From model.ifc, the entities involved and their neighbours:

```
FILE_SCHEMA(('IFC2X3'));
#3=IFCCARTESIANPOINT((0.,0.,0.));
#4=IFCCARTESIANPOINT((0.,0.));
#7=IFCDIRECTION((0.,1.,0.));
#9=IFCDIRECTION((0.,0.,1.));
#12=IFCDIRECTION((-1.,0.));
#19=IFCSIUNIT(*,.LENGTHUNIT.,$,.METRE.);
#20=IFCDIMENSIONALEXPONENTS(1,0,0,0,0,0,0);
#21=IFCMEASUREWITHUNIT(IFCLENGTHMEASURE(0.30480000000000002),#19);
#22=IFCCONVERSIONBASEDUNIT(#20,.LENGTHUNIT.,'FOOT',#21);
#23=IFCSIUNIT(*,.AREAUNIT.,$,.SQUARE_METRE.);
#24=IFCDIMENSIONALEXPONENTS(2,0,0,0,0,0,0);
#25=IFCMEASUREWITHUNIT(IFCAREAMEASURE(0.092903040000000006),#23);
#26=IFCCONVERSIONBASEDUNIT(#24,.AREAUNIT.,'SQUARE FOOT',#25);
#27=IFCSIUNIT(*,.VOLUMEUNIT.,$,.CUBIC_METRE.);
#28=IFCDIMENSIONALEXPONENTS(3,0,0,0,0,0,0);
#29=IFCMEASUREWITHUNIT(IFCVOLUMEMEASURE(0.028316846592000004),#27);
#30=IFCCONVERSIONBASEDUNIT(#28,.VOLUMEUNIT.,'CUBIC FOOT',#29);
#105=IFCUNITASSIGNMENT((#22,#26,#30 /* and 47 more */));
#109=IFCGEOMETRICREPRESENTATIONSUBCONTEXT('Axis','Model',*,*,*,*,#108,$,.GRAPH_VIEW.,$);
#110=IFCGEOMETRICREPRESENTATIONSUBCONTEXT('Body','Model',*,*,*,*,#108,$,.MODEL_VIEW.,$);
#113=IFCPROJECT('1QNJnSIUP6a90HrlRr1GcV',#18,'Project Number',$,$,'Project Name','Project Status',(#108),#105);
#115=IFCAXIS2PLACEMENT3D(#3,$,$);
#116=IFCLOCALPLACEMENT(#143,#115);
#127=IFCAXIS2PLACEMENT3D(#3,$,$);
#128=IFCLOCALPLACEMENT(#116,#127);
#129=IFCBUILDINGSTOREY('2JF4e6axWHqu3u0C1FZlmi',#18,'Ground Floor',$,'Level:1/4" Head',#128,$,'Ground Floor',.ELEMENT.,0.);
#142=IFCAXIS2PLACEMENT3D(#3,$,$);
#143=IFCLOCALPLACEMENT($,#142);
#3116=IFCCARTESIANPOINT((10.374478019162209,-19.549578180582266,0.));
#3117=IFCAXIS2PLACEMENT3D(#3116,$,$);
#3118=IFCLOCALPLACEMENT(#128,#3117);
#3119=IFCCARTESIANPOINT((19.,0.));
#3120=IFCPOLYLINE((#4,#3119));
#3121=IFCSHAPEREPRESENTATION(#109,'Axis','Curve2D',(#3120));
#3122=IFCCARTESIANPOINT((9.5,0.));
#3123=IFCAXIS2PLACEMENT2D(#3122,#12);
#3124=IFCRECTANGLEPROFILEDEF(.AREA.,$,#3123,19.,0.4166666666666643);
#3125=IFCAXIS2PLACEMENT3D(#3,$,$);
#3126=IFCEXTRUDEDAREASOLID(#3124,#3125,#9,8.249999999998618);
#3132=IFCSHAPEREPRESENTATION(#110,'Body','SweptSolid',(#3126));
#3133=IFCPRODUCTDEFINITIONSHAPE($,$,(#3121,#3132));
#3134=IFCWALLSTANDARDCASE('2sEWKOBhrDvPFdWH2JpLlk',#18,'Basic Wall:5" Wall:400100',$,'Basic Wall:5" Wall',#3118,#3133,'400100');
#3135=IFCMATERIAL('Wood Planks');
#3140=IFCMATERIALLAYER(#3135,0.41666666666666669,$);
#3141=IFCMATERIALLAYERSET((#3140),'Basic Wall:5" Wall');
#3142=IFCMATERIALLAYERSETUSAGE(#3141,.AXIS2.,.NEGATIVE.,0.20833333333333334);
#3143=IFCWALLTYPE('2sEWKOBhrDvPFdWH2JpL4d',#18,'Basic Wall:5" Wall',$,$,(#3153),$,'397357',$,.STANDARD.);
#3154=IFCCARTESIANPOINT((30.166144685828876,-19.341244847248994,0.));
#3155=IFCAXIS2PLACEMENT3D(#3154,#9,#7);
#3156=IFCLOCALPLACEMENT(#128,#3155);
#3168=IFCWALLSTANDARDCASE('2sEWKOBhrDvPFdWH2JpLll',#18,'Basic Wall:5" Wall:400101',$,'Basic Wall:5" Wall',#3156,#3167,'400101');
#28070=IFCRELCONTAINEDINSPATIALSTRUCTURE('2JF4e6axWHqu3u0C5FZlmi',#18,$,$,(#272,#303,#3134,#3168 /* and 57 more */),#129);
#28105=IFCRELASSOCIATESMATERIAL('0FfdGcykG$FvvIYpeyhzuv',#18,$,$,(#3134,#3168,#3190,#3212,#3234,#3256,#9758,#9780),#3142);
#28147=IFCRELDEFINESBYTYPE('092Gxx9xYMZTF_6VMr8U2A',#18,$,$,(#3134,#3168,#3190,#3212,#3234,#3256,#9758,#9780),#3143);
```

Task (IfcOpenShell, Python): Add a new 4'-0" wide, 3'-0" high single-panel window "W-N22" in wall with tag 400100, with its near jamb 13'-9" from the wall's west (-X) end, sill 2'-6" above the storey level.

```python
import numpy as np
import ifcopenshell
import ifcopenshell.api.feature
import ifcopenshell.api.geometry
import ifcopenshell.api.root
import ifcopenshell.api.spatial
import ifcopenshell.api.type
import ifcopenshell.geom
import ifcopenshell.util.element
import ifcopenshell.util.placement
import ifcopenshell.util.representation
import ifcopenshell.util.shape
import ifcopenshell.util.unit

model = ifcopenshell.open("model.ifc")
unit_scale = ifcopenshell.util.unit.calculate_unit_scale(model)
settings = ifcopenshell.geom.settings()


def volume(element):
    """Net volume in cubic metres, openings subtracted."""
    shape = ifcopenshell.geom.create_shape(settings, element)
    return ifcopenshell.util.shape.get_volume(shape.geometry)


wall = model.by_id(3134)
storey = ifcopenshell.util.element.get_container(wall, ifc_class="IfcBuildingStorey")
context = ifcopenshell.util.representation.get_context(model, "Model", "Body", "MODEL_VIEW")
before = volume(wall)

width, height, from_end, sill = 1.2192, 0.9144, 4.191, 0.762  # metres

# The wall runs along its own X axis, and the end named is its -X end.
wall_shape = ifcopenshell.geom.create_shape(settings, wall)
x, y, z = ifcopenshell.util.shape.get_vertices(wall_shape.geometry).T
start = x.min() + from_end
face, thickness = float(y.min()), float(y.max() - y.min())
wall_matrix = ifcopenshell.util.placement.get_local_placement(wall.ObjectPlacement)
level = ifcopenshell.util.placement.get_local_placement(storey.ObjectPlacement)[2, 3]


def in_wall(x, y):
    """Placement at x, y metres in the wall's axes, at sill height."""
    matrix = wall_matrix.copy()
    matrix[:, 3] = wall_matrix @ np.array([x / unit_scale, y / unit_scale, 0.0, 1.0])
    matrix[2, 3] = level + sill / unit_scale
    return matrix


# Opening: a box that overshoots both wall faces by 50 mm.
opening = ifcopenshell.api.root.create_entity(model, ifc_class="IfcOpeningElement")
box = ifcopenshell.api.geometry.add_wall_representation(
    model, context=context, length=width, height=height, thickness=thickness + 0.1
)
ifcopenshell.api.geometry.assign_representation(model, product=opening, representation=box)
ifcopenshell.api.geometry.edit_object_placement(model, product=opening, matrix=in_wall(start, face - 0.05), is_si=False)
ifcopenshell.api.feature.add_feature(model, feature=opening, element=wall)

window = ifcopenshell.api.root.create_entity(model, ifc_class="IfcWindow", name="W-N22")
window.OverallWidth, window.OverallHeight = width / unit_scale, height / unit_scale
body = ifcopenshell.api.geometry.add_window_representation(
    model,
    context=context,
    overall_width=window.OverallWidth,
    overall_height=window.OverallHeight,
    partition_type="SINGLE_PANEL",
)
ifcopenshell.api.geometry.assign_representation(model, product=window, representation=body)
ifcopenshell.api.spatial.assign_container(model, products=[window], relating_structure=storey)
fills = ifcopenshell.api.feature.add_filling(model, opening=opening, element=window)
fills.OwnerHistory = window.OwnerHistory  # required in IFC2X3

# IFC2X3 keeps the operation on the window style.
style = ifcopenshell.api.root.create_entity(model, ifc_class="IfcWindowStyle", name="W-N22")
style.OperationType, style.ConstructionType = "SINGLE_PANEL", "NOTDEFINED"
style.ParameterTakesPrecedence = style.Sizeable = False
ifcopenshell.api.type.assign_type(model, related_objects=[window], relating_type=style)

# Centre the window in the wall's thickness.
ifcopenshell.api.geometry.edit_object_placement(model, product=window, matrix=in_wall(start, face), is_si=False)
window_shape = ifcopenshell.geom.create_shape(settings, window)
depth = ifcopenshell.util.shape.get_vertices(window_shape.geometry)[:, 1]
offset = face + thickness / 2 - (depth.min() + depth.max()) / 2
ifcopenshell.api.geometry.edit_object_placement(model, product=window, matrix=in_wall(start, offset), is_si=False)

after = volume(wall)

print(f"wall volume {before:.3f} -> {after:.3f} m3")

model.write("model_updated.ifc")
```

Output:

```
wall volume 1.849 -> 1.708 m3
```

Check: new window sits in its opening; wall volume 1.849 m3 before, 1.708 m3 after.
